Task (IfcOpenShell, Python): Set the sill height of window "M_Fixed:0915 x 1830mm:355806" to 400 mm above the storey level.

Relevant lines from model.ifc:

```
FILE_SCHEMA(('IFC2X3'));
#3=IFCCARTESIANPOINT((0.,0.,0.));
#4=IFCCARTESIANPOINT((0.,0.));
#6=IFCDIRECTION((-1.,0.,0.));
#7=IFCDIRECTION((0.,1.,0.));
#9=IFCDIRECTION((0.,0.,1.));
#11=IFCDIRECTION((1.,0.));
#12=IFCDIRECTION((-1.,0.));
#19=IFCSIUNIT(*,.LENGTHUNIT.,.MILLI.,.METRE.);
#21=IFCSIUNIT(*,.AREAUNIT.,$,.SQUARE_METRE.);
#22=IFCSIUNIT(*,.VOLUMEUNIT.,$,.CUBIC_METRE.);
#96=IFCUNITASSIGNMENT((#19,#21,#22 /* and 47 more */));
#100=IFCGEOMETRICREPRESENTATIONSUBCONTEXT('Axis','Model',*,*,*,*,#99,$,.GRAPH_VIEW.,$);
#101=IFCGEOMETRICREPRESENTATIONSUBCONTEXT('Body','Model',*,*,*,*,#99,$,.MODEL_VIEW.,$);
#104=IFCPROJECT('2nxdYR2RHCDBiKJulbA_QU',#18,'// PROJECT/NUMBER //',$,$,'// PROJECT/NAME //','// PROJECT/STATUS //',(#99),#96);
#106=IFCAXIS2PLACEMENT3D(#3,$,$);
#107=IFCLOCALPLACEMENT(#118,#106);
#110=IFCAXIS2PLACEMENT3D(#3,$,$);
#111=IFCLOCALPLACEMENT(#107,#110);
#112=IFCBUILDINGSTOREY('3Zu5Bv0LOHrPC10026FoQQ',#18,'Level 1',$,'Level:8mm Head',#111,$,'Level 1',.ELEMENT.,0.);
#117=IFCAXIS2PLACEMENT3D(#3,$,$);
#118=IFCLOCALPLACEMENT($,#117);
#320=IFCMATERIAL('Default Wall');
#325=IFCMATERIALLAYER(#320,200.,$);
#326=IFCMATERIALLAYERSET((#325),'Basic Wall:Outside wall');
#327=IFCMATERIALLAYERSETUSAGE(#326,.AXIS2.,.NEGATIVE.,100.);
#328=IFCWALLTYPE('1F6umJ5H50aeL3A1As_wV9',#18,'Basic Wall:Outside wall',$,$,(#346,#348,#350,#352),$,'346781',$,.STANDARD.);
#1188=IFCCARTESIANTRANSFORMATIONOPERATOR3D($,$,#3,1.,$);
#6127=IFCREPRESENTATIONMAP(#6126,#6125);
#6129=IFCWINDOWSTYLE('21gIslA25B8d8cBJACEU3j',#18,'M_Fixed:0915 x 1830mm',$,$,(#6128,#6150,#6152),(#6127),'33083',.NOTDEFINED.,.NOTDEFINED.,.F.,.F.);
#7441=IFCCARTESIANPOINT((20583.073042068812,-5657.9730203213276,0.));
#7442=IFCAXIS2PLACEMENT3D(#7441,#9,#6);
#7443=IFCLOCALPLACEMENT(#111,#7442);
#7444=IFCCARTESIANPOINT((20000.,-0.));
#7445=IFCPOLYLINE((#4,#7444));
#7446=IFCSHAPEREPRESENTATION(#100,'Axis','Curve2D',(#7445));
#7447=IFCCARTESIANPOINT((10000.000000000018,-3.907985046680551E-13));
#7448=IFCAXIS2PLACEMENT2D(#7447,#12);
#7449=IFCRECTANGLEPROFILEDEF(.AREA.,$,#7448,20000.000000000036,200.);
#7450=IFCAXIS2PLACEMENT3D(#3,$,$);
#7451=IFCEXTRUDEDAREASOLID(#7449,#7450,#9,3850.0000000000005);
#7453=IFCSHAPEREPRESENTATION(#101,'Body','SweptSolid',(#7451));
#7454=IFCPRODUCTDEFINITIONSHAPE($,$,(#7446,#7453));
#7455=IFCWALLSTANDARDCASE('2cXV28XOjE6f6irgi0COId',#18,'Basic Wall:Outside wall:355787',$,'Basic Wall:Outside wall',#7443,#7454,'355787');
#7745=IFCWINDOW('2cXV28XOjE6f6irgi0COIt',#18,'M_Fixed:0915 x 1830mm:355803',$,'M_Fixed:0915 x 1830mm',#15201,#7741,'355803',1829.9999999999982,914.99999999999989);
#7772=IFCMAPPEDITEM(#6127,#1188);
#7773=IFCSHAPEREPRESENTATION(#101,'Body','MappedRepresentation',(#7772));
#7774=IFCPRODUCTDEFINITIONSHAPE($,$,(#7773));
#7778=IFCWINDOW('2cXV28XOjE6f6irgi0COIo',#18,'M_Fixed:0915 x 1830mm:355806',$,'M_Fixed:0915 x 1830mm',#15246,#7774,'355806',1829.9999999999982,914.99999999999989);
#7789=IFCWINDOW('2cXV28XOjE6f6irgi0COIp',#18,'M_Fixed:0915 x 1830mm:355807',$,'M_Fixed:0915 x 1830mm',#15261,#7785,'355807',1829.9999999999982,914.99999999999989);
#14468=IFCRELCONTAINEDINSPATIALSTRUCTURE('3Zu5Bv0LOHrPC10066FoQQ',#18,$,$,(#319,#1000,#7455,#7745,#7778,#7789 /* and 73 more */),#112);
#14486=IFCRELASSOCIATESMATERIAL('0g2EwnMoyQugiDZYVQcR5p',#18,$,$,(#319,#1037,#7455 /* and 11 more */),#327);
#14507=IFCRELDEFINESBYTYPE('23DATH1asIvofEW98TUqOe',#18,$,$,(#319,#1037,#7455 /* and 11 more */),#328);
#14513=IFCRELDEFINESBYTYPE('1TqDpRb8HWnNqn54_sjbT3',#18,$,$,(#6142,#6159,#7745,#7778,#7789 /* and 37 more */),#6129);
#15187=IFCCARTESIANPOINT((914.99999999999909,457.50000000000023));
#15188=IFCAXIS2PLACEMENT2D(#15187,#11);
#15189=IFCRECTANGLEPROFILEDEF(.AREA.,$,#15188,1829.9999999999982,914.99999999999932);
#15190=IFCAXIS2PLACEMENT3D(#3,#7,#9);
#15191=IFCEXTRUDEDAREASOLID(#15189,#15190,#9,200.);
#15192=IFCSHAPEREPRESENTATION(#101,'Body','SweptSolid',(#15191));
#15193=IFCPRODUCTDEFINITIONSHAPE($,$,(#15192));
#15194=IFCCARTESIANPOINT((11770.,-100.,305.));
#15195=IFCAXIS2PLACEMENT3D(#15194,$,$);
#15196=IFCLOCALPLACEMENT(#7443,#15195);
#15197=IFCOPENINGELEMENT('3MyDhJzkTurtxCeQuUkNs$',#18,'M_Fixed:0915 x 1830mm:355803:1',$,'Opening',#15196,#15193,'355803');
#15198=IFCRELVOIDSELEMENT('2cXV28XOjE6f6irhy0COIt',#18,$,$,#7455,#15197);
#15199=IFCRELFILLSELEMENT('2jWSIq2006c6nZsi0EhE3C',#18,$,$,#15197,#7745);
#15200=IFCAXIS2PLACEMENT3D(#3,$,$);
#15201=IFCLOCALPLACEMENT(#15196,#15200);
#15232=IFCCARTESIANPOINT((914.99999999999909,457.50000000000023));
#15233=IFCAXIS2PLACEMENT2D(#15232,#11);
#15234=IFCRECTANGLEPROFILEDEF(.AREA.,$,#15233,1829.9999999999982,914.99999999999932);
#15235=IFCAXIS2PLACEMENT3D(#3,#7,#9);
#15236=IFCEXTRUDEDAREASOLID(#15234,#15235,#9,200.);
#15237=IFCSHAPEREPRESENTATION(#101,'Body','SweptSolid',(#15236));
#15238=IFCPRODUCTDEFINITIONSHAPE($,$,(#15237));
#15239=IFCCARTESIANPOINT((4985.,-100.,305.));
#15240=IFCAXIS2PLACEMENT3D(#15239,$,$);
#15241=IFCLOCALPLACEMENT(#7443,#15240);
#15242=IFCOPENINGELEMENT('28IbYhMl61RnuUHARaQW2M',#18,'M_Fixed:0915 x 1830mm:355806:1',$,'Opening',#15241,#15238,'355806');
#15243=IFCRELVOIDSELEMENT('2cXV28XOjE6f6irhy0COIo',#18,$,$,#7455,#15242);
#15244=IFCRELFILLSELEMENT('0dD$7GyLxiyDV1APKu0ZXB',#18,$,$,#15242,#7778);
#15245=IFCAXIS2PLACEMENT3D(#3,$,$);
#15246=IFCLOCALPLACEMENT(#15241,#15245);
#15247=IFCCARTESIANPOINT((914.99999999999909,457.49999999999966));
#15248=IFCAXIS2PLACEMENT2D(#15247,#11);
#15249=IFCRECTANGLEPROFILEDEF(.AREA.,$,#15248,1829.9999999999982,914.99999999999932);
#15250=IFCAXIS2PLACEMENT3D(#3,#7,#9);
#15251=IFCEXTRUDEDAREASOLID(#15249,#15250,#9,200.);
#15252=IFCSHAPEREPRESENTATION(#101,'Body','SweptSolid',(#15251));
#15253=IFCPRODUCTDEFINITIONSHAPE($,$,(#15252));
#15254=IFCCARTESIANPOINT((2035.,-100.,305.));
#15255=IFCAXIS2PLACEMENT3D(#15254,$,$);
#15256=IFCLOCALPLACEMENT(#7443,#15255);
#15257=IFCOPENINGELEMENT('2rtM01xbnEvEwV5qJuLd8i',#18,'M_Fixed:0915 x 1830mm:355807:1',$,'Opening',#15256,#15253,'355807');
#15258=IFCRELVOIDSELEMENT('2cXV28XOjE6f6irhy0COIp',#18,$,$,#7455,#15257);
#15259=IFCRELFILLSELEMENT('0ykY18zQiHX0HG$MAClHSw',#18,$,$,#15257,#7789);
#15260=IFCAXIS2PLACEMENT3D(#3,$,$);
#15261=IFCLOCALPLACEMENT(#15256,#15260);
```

```python
import numpy as np
import ifcopenshell
import ifcopenshell.api.geometry
import ifcopenshell.geom
import ifcopenshell.util.element
import ifcopenshell.util.placement
import ifcopenshell.util.shape
import ifcopenshell.util.unit

model = ifcopenshell.open("model.ifc")
unit_scale = ifcopenshell.util.unit.calculate_unit_scale(model)

window = model.by_guid("2cXV28XOjE6f6irgi0COIo")
opening = window.FillsVoids[0].RelatingOpeningElement
storey = ifcopenshell.util.element.get_container(window, ifc_class="IfcBuildingStorey")
level = ifcopenshell.util.placement.get_local_placement(storey.ObjectPlacement)[2, 3]

# The opening's origin need not be at the sill, so measure its lowest point.
shape = ifcopenshell.geom.create_shape(ifcopenshell.geom.settings(), opening)
bottom = ifcopenshell.util.shape.get_shape_bottom_elevation(shape, shape.geometry) / unit_scale
dz = level + 0.4 / unit_scale - bottom

shift = np.array([0.0, 0.0, dz])
# The window is placed relative to its opening, so it follows when the opening moves.
matrix = ifcopenshell.util.placement.get_local_placement(opening.ObjectPlacement)
matrix[:3, 3] += shift
ifcopenshell.api.geometry.edit_object_placement(
    model, product=opening, matrix=matrix, is_si=False, should_transform_children=True
)

print(f"moved by {dz * unit_scale:+.3f} m")

model.write("model_rev.ifc")
```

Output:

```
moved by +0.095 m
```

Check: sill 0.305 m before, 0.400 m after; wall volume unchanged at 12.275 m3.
